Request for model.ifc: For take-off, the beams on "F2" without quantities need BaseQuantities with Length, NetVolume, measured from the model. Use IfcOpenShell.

First a look at what the model holds.

```python
import ifcopenshell
import ifcopenshell.util.element
import ifcopenshell.util.unit

model = ifcopenshell.open("model.ifc")
print(model.schema)
for unit_type in ("LENGTHUNIT", "AREAUNIT", "VOLUMEUNIT"):
    print(unit_type, ifcopenshell.util.unit.calculate_unit_scale(model, unit_type))
storey = next(s for s in model.by_type("IfcBuildingStorey") if s.Name == "F2")
beams = [e for e in ifcopenshell.util.element.get_decomposition(storey) if e.is_a("IfcBeam")]
for e in sorted(beams, key=lambda e: e.id()):
    print(e.id(), e.is_a(), e.Name, list(ifcopenshell.util.element.get_psets(e, qtos_only=True)), sep=" | ")
```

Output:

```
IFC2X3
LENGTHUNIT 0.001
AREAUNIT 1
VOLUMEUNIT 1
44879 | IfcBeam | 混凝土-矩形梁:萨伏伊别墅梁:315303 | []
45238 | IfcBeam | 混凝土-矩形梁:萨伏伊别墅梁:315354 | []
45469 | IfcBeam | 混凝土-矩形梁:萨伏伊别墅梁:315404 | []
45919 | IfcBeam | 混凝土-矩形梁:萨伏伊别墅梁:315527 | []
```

```python
import ifcopenshell
import ifcopenshell.api.pset
import ifcopenshell.geom
import ifcopenshell.util.element
import ifcopenshell.util.shape
import ifcopenshell.util.unit

model = ifcopenshell.open("model.ifc")
unit_scale = ifcopenshell.util.unit.calculate_unit_scale(model)
volume_scale = ifcopenshell.util.unit.calculate_unit_scale(model, "VOLUMEUNIT")
settings = ifcopenshell.geom.settings()

storey = next(s for s in model.by_type("IfcBuildingStorey") if s.Name == "F2")
beams = [e for e in ifcopenshell.util.element.get_decomposition(storey) if e.is_a("IfcBeam")]

for e in sorted(beams, key=lambda e: e.id()):
    if ifcopenshell.util.element.get_psets(e, qtos_only=True, should_inherit=False):
        continue
    # Geometry comes back in metres, in the element's own axes.
    shape = ifcopenshell.geom.create_shape(settings, e)
    values = {
        "Length": ifcopenshell.util.shape.get_max_xyz(shape.geometry) / unit_scale,
        "NetVolume": ifcopenshell.util.shape.get_volume(shape.geometry) / volume_scale,
    }
    qto = ifcopenshell.api.pset.add_qto(model, product=e, name="BaseQuantities")
    ifcopenshell.api.pset.edit_qto(model, qto=qto, properties=values)
    print(e.id(), {k: round(v, 3) for k, v in values.items()})

model.write("model_updated.ifc")
```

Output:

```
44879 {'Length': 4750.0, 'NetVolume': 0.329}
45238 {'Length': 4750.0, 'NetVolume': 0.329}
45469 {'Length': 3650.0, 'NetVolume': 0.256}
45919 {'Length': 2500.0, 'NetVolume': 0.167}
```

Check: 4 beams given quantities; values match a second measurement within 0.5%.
